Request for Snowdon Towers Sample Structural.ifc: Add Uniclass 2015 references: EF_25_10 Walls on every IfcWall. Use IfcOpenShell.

First a look at what the model holds.

```python
import ifcopenshell

model = ifcopenshell.open("Snowdon Towers Sample Structural.ifc")
print(model.schema)
print("classifications:", [c.Name for c in model.by_type("IfcClassification")])
for ifc_class in ("IfcDoor", "IfcRoof", "IfcStair", "IfcWall", "IfcWindow"):
    print(ifc_class, len(model.by_type(ifc_class)))
```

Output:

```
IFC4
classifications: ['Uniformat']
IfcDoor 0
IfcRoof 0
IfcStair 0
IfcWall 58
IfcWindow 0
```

```python
import ifcopenshell
import ifcopenshell.api.classification

model = ifcopenshell.open("Snowdon Towers Sample Structural.ifc")

system = ifcopenshell.api.classification.add_classification(model, classification="Uniclass 2015")

codes = {
    "IfcWall": ("EF_25_10", "Walls"),
}
for ifc_class, (code, name) in codes.items():
    products = model.by_type(ifc_class)
    ifcopenshell.api.classification.add_reference(
        model, products=products, classification=system, identification=code, name=name
    )
    print(code, len(products))

model.write("Snowdon Towers Sample Structural_v2.ifc")
```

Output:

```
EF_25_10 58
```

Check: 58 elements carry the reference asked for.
